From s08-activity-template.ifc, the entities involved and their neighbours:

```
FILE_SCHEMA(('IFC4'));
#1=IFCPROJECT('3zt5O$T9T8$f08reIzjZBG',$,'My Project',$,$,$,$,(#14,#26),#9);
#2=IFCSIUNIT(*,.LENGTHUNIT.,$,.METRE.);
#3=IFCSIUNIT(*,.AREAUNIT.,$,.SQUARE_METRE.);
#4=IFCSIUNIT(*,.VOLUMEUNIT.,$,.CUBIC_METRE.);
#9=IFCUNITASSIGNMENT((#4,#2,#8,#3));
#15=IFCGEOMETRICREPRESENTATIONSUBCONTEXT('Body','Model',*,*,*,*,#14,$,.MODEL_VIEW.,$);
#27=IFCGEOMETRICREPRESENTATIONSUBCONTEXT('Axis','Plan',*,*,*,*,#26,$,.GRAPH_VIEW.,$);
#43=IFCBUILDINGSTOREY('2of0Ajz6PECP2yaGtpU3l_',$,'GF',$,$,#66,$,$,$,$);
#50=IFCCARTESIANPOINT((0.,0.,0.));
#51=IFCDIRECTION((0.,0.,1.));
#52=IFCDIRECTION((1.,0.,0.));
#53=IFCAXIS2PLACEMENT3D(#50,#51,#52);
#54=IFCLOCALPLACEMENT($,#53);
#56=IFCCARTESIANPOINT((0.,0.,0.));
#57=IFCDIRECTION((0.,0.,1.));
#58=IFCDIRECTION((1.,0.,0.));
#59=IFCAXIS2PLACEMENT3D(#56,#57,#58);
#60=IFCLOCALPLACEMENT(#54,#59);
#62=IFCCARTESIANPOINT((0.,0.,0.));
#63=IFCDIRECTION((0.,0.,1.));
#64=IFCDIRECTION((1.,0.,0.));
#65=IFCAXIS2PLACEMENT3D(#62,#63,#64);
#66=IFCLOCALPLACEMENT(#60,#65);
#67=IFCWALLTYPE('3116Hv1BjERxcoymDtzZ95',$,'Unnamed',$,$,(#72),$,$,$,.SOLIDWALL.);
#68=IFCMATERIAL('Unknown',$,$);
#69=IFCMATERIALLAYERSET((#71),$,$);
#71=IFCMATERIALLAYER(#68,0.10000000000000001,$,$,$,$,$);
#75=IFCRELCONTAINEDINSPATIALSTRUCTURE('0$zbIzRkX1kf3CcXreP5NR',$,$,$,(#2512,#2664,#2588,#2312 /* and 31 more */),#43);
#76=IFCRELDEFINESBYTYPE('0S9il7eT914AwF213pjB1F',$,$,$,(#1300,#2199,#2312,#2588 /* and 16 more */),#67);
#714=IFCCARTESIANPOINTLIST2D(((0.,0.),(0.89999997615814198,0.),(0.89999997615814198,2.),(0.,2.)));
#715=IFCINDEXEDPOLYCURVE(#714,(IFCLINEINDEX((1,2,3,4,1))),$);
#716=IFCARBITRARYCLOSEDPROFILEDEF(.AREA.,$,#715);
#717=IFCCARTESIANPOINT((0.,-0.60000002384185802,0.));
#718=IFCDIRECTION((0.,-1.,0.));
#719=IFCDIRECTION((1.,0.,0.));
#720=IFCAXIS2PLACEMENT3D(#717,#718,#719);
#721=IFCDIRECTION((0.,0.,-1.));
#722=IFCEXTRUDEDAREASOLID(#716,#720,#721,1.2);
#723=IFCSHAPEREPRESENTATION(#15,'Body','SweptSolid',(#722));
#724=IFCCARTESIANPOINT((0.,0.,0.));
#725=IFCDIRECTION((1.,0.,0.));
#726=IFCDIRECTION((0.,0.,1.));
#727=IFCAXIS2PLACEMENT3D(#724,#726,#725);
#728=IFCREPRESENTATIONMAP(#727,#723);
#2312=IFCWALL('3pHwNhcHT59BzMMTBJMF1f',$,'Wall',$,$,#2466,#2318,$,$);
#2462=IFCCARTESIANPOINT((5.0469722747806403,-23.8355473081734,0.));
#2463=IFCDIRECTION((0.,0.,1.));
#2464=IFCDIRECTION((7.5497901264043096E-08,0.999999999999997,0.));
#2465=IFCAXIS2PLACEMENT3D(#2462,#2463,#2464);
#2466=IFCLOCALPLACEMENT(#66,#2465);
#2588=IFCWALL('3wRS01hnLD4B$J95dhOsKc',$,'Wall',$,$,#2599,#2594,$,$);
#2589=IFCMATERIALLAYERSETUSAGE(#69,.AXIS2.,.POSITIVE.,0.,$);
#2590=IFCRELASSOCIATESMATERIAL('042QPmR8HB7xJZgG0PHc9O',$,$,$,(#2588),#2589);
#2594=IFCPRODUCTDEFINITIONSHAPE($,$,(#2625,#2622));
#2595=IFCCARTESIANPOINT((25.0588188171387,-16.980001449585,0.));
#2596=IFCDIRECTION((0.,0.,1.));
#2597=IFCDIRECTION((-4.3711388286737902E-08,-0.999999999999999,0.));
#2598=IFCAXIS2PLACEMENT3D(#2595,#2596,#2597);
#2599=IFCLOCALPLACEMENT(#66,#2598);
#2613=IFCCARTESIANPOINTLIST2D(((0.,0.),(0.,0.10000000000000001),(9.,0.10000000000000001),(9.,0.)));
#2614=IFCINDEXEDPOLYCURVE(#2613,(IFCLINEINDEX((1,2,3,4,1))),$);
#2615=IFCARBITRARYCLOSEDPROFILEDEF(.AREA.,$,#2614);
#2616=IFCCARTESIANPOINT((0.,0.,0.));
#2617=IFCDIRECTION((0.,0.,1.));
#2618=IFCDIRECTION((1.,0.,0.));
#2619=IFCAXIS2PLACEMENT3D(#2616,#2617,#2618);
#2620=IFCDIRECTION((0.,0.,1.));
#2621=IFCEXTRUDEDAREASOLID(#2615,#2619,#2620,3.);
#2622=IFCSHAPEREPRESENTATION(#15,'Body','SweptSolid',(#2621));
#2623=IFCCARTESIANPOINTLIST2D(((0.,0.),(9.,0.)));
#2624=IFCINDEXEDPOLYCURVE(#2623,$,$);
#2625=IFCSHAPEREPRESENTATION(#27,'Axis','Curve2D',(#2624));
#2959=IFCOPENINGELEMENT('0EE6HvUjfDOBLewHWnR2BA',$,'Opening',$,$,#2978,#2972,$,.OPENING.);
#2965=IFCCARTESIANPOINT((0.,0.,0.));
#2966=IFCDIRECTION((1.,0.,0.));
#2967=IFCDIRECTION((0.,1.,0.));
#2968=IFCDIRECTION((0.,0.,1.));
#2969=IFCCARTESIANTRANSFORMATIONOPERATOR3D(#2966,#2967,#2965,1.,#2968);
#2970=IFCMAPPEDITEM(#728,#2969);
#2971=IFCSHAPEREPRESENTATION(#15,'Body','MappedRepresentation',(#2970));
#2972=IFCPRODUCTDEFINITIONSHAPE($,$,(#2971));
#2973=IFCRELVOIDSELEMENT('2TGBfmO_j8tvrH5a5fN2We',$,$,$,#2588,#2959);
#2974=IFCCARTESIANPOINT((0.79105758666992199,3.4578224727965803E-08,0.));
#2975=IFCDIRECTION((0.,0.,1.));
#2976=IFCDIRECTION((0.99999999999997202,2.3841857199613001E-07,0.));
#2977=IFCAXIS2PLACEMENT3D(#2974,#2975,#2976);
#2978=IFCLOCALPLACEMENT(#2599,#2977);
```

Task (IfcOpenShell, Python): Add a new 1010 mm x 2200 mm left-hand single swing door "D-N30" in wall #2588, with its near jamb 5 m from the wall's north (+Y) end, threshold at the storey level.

```python
import numpy as np
import ifcopenshell
import ifcopenshell.api.feature
import ifcopenshell.api.geometry
import ifcopenshell.api.root
import ifcopenshell.api.spatial
import ifcopenshell.geom
import ifcopenshell.util.element
import ifcopenshell.util.placement
import ifcopenshell.util.representation
import ifcopenshell.util.shape
import ifcopenshell.util.unit

model = ifcopenshell.open("s08-activity-template.ifc")
unit_scale = ifcopenshell.util.unit.calculate_unit_scale(model)
settings = ifcopenshell.geom.settings()


def volume(element):
    """Net volume in cubic metres, openings subtracted."""
    shape = ifcopenshell.geom.create_shape(settings, element)
    return ifcopenshell.util.shape.get_volume(shape.geometry)


wall = model.by_guid("3wRS01hnLD4B$J95dhOsKc")
storey = ifcopenshell.util.element.get_container(wall, ifc_class="IfcBuildingStorey")
context = ifcopenshell.util.representation.get_context(model, "Model", "Body", "MODEL_VIEW")
before = volume(wall)

width, height, from_end, sill = 1.01, 2.2, 5, 0.0  # metres

# The wall runs along its own X axis, and the end named is its -X end.
wall_shape = ifcopenshell.geom.create_shape(settings, wall)
x, y, z = ifcopenshell.util.shape.get_vertices(wall_shape.geometry).T
start = x.min() + from_end
face, thickness = float(y.min()), float(y.max() - y.min())
wall_matrix = ifcopenshell.util.placement.get_local_placement(wall.ObjectPlacement)
level = ifcopenshell.util.placement.get_local_placement(storey.ObjectPlacement)[2, 3]


def in_wall(x, y):
    """Placement at x, y metres in the wall's axes, at sill height."""
    matrix = wall_matrix.copy()
    matrix[:, 3] = wall_matrix @ np.array([x / unit_scale, y / unit_scale, 0.0, 1.0])
    matrix[2, 3] = level + sill / unit_scale
    return matrix


# Opening: a box that overshoots both wall faces by 50 mm.
opening = ifcopenshell.api.root.create_entity(model, ifc_class="IfcOpeningElement", predefined_type="OPENING")
box = ifcopenshell.api.geometry.add_wall_representation(
    model, context=context, length=width, height=height, thickness=thickness + 0.1
)
ifcopenshell.api.geometry.assign_representation(model, product=opening, representation=box)
ifcopenshell.api.geometry.edit_object_placement(model, product=opening, matrix=in_wall(start, face - 0.05), is_si=False)
ifcopenshell.api.feature.add_feature(model, feature=opening, element=wall)

door = ifcopenshell.api.root.create_entity(model, ifc_class="IfcDoor", name="D-N30", predefined_type="DOOR")
door.OverallWidth, door.OverallHeight = width / unit_scale, height / unit_scale
door.OperationType = "SINGLE_SWING_LEFT"
body = ifcopenshell.api.geometry.add_door_representation(
    model,
    context=context,
    overall_width=door.OverallWidth,
    overall_height=door.OverallHeight,
    operation_type="SINGLE_SWING_LEFT",
    lining_properties={"LiningDepth": thickness / unit_scale, "ThresholdDepth": thickness / unit_scale},
)
ifcopenshell.api.geometry.assign_representation(model, product=door, representation=body)
ifcopenshell.api.spatial.assign_container(model, products=[door], relating_structure=storey)
ifcopenshell.api.feature.add_filling(model, opening=opening, element=door)

# The lining spans the wall, so the door starts at the wall face.
ifcopenshell.api.geometry.edit_object_placement(model, product=door, matrix=in_wall(start, face), is_si=False)

after = volume(wall)

print(f"wall volume {before:.3f} -> {after:.3f} m3")

model.write("s08-activity-template_edited.ifc")
```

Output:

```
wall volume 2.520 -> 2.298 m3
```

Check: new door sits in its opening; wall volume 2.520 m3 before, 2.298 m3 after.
